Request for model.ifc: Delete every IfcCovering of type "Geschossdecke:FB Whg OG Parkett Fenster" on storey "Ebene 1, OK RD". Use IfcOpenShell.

First a look at what the model holds.

```python
import ifcopenshell
import ifcopenshell.util.element

model = ifcopenshell.open("model.ifc")
print(model.schema)
storey = next(s for s in model.by_type("IfcBuildingStorey") if s.Name == "Ebene 1, OK RD")
coverings = [e for e in ifcopenshell.util.element.get_decomposition(storey) if e.is_a("IfcCovering")]
seen = {}
for e in coverings:
    element_type = ifcopenshell.util.element.get_type(e)
    name = element_type.Name if element_type not in (None, e) else None
    seen[name] = seen.get(name, 0) + 1
for name, count in sorted(seen.items(), key=str):
    print(count, "x", name)
```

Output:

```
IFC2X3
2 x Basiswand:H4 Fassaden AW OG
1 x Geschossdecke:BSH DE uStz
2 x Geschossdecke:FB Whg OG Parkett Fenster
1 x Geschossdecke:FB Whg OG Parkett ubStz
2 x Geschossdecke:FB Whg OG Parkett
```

```python
import ifcopenshell
import ifcopenshell.api.root
import ifcopenshell.util.element

model = ifcopenshell.open("model.ifc")

storey = next(s for s in model.by_type("IfcBuildingStorey") if s.Name == "Ebene 1, OK RD")
coverings = [e for e in ifcopenshell.util.element.get_decomposition(storey) if e.is_a("IfcCovering")]
targets = [e for e in coverings if (t := ifcopenshell.util.element.get_type(e)) not in (None, e) and t.Name == "Geschossdecke:FB Whg OG Parkett Fenster"]

for e in targets:
    ifcopenshell.api.root.remove_product(model, product=e)
print(len(targets), "removed")

model.write("model_updated.ifc")
```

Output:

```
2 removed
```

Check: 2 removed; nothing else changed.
